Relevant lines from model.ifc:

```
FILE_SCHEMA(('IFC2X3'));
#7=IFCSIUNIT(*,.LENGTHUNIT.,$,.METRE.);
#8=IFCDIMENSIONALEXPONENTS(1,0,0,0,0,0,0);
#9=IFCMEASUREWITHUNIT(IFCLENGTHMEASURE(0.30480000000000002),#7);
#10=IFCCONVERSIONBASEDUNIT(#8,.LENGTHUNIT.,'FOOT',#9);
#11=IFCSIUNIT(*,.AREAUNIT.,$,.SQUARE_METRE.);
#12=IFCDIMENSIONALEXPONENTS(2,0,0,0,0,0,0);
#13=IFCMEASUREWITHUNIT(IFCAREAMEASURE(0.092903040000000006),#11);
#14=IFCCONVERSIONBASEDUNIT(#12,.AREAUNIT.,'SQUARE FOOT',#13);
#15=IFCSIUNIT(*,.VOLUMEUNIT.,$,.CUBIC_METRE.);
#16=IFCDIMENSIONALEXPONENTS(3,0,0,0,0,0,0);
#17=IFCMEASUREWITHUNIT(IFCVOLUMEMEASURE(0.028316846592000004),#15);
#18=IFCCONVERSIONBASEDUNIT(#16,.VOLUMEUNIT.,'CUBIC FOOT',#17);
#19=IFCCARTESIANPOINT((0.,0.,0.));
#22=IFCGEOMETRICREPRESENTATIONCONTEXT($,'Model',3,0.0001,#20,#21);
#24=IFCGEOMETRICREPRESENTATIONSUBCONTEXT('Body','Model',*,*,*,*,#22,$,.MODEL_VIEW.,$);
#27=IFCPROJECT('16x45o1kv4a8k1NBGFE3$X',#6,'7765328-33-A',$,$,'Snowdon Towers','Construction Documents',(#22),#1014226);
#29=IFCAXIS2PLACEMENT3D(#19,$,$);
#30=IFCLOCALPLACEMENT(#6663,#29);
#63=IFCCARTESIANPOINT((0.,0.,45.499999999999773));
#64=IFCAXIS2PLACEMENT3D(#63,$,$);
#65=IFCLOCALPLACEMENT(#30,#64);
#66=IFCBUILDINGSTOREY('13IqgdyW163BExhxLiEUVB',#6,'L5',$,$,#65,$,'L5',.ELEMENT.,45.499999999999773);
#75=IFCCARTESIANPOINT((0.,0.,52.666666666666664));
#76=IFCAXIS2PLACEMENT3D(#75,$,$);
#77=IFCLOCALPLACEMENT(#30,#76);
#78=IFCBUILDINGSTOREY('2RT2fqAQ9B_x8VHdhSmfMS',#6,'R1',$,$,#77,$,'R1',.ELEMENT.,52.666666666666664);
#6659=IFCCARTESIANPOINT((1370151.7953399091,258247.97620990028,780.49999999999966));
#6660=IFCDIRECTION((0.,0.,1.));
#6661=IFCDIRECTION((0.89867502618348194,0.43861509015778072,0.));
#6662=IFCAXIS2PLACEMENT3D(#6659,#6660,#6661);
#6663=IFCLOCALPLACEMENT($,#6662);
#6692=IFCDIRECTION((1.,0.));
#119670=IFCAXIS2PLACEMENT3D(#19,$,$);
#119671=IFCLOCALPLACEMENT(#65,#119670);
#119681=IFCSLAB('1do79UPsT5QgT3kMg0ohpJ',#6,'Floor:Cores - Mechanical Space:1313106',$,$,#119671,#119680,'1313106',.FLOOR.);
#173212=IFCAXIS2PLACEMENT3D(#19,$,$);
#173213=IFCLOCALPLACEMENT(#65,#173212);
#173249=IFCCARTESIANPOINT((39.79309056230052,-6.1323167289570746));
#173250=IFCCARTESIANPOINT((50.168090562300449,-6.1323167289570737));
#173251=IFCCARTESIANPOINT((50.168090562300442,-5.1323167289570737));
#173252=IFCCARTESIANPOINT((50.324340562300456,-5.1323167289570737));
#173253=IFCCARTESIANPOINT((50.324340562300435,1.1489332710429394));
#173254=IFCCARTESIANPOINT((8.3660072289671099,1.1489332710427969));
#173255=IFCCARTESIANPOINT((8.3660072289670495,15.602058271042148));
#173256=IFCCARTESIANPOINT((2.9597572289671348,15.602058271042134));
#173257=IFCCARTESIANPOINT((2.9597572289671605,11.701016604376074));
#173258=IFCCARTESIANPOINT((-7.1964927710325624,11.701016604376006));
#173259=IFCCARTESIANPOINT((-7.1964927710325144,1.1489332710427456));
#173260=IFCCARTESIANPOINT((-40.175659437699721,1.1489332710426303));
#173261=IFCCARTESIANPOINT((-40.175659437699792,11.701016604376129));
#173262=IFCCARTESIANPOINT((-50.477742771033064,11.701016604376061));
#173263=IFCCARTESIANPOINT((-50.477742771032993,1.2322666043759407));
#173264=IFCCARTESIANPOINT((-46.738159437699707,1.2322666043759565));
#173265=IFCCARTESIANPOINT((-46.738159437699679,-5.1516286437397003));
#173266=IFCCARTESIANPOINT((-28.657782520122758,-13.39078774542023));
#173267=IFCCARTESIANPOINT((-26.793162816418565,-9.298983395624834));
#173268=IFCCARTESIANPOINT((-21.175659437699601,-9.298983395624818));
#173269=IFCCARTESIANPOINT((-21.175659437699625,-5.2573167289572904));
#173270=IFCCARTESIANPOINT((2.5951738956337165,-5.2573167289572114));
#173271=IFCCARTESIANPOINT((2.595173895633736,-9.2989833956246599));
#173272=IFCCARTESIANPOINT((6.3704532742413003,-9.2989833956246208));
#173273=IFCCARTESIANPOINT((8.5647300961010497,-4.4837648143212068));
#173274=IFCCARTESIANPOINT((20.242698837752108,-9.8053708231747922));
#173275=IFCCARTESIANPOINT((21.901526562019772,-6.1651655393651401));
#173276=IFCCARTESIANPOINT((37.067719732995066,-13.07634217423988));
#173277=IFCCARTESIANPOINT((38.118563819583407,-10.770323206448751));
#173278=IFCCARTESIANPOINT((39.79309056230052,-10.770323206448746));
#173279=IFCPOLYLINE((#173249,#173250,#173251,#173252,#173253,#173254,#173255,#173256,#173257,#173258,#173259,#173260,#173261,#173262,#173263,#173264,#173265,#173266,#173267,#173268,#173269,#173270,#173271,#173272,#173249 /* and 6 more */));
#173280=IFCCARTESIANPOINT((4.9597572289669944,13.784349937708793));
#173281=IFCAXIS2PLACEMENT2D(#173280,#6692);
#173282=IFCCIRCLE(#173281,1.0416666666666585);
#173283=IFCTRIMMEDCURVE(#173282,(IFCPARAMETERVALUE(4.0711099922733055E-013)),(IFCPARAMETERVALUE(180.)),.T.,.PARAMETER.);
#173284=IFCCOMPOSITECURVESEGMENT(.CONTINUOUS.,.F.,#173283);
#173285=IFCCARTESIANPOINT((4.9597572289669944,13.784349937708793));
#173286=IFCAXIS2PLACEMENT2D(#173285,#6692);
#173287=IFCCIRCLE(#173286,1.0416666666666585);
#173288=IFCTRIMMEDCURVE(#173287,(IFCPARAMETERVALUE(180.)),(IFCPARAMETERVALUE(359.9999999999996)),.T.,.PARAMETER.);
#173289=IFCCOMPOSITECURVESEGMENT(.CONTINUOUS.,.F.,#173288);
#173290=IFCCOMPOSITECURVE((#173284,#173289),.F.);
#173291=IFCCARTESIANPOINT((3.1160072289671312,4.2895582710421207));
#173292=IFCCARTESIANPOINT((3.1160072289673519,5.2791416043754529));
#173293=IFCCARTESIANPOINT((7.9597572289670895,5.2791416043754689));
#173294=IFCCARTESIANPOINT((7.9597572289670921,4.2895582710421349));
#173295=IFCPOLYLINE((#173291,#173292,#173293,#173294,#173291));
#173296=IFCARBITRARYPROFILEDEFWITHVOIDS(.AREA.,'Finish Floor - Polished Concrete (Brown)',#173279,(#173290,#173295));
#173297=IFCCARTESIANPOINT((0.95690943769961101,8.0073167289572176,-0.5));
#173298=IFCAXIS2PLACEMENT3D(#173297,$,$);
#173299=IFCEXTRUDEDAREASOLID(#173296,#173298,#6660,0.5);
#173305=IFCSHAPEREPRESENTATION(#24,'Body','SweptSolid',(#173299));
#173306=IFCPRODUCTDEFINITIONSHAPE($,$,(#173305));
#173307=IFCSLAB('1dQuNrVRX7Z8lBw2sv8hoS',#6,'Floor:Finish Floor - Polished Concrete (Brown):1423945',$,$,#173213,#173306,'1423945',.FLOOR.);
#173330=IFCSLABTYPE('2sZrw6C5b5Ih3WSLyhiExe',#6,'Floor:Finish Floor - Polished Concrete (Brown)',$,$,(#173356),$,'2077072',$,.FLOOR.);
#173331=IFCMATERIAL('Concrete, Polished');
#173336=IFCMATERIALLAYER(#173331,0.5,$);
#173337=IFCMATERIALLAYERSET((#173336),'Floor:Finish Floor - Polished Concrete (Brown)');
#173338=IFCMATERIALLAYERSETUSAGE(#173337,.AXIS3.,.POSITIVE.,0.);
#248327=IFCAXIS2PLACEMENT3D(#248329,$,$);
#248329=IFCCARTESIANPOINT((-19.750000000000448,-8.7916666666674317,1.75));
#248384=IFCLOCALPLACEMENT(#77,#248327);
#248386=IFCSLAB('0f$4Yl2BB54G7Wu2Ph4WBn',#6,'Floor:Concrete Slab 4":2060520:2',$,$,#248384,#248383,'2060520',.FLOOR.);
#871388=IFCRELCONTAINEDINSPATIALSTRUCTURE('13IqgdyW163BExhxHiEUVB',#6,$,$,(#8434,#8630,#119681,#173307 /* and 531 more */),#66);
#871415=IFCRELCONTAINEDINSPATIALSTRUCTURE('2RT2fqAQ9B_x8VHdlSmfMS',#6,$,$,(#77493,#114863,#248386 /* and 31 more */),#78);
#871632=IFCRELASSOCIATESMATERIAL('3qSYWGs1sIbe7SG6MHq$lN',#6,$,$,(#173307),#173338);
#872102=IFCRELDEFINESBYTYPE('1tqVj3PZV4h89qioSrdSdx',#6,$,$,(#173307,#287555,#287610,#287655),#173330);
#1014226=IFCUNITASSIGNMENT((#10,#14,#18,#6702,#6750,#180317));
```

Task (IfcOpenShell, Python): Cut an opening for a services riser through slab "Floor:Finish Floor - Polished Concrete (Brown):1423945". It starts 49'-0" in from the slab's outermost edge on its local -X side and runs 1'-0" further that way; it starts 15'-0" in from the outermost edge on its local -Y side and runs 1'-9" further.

```python
import numpy as np
import ifcopenshell
import ifcopenshell.api.feature
import ifcopenshell.api.geometry
import ifcopenshell.api.root
import ifcopenshell.geom
import ifcopenshell.util.placement
import ifcopenshell.util.representation
import ifcopenshell.util.shape
import ifcopenshell.util.unit

model = ifcopenshell.open("model.ifc")
unit_scale = ifcopenshell.util.unit.calculate_unit_scale(model)
settings = ifcopenshell.geom.settings()


def volume(element):
    """Net volume in cubic metres, openings subtracted."""
    shape = ifcopenshell.geom.create_shape(settings, element)
    return ifcopenshell.util.shape.get_volume(shape.geometry)


slab = model.by_guid("1dQuNrVRX7Z8lBw2sv8hoS")
before = volume(slab)

# Extent in the slab's own axes, in metres. The edges named are its -X and -Y sides.
slab_shape = ifcopenshell.geom.create_shape(settings, slab)
vertices = ifcopenshell.util.shape.get_vertices(slab_shape.geometry)
x_min, y_min, bottom = vertices.min(axis=0)
top = vertices[:, 2].max()

opening = ifcopenshell.api.root.create_entity(model, ifc_class="IfcOpeningElement", name="Services riser opening")
context = ifcopenshell.util.representation.get_context(model, "Model", "Body", "MODEL_VIEW")
width, depth = 0.3048, 0.5334
outline = [(0.0, 0.0), (width, 0.0), (width, depth), (0.0, depth), (0.0, 0.0)]
# Overshoot both faces by 50 mm so the cut is clean.
shape = ifcopenshell.api.geometry.add_slab_representation(
    model, context=context, depth=top - bottom + 0.1, polyline=outline
)
ifcopenshell.api.geometry.assign_representation(model, product=opening, representation=shape)

matrix = ifcopenshell.util.placement.get_local_placement(slab.ObjectPlacement)
matrix[:, 3] = matrix @ np.append(np.array([x_min + 14.9352, y_min + 4.572, bottom - 0.05]) / unit_scale, 1.0)
ifcopenshell.api.geometry.edit_object_placement(model, product=opening, matrix=matrix, is_si=False)
ifcopenshell.api.feature.add_feature(model, feature=opening, element=slab)

after = volume(slab)

print(f"slab volume {before:.3f} -> {after:.3f} m3")

model.write("model_updated.ifc")
```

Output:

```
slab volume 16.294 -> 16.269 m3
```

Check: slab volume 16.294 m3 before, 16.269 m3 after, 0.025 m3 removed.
